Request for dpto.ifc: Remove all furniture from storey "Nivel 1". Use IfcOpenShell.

First a look at what the model holds.

```python
import ifcopenshell
import ifcopenshell.util.element

model = ifcopenshell.open("dpto.ifc")
print(model.schema)
storey = next(s for s in model.by_type("IfcBuildingStorey") if s.Name == "Nivel 1")
furniture = [e for e in ifcopenshell.util.element.get_decomposition(storey) if e.is_a("IfcFurnishingElement")]
seen = {}
for e in furniture:
    element_type = ifcopenshell.util.element.get_type(e)
    name = element_type.Name if element_type not in (None, e) else None
    seen[name] = seen.get(name, 0) + 1
for name, count in sorted(seen.items(), key=str):
    print(count, "x", name)
```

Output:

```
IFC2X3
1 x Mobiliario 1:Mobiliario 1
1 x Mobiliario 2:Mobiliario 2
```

```python
import ifcopenshell
import ifcopenshell.api.root
import ifcopenshell.util.element

model = ifcopenshell.open("dpto.ifc")

storey = next(s for s in model.by_type("IfcBuildingStorey") if s.Name == "Nivel 1")
furniture = [e for e in ifcopenshell.util.element.get_decomposition(storey) if e.is_a("IfcFurnishingElement")]

for e in furniture:
    ifcopenshell.api.root.remove_product(model, product=e)
print(len(furniture), "removed")

model.write("dpto-out.ifc")
```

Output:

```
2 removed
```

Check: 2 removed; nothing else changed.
